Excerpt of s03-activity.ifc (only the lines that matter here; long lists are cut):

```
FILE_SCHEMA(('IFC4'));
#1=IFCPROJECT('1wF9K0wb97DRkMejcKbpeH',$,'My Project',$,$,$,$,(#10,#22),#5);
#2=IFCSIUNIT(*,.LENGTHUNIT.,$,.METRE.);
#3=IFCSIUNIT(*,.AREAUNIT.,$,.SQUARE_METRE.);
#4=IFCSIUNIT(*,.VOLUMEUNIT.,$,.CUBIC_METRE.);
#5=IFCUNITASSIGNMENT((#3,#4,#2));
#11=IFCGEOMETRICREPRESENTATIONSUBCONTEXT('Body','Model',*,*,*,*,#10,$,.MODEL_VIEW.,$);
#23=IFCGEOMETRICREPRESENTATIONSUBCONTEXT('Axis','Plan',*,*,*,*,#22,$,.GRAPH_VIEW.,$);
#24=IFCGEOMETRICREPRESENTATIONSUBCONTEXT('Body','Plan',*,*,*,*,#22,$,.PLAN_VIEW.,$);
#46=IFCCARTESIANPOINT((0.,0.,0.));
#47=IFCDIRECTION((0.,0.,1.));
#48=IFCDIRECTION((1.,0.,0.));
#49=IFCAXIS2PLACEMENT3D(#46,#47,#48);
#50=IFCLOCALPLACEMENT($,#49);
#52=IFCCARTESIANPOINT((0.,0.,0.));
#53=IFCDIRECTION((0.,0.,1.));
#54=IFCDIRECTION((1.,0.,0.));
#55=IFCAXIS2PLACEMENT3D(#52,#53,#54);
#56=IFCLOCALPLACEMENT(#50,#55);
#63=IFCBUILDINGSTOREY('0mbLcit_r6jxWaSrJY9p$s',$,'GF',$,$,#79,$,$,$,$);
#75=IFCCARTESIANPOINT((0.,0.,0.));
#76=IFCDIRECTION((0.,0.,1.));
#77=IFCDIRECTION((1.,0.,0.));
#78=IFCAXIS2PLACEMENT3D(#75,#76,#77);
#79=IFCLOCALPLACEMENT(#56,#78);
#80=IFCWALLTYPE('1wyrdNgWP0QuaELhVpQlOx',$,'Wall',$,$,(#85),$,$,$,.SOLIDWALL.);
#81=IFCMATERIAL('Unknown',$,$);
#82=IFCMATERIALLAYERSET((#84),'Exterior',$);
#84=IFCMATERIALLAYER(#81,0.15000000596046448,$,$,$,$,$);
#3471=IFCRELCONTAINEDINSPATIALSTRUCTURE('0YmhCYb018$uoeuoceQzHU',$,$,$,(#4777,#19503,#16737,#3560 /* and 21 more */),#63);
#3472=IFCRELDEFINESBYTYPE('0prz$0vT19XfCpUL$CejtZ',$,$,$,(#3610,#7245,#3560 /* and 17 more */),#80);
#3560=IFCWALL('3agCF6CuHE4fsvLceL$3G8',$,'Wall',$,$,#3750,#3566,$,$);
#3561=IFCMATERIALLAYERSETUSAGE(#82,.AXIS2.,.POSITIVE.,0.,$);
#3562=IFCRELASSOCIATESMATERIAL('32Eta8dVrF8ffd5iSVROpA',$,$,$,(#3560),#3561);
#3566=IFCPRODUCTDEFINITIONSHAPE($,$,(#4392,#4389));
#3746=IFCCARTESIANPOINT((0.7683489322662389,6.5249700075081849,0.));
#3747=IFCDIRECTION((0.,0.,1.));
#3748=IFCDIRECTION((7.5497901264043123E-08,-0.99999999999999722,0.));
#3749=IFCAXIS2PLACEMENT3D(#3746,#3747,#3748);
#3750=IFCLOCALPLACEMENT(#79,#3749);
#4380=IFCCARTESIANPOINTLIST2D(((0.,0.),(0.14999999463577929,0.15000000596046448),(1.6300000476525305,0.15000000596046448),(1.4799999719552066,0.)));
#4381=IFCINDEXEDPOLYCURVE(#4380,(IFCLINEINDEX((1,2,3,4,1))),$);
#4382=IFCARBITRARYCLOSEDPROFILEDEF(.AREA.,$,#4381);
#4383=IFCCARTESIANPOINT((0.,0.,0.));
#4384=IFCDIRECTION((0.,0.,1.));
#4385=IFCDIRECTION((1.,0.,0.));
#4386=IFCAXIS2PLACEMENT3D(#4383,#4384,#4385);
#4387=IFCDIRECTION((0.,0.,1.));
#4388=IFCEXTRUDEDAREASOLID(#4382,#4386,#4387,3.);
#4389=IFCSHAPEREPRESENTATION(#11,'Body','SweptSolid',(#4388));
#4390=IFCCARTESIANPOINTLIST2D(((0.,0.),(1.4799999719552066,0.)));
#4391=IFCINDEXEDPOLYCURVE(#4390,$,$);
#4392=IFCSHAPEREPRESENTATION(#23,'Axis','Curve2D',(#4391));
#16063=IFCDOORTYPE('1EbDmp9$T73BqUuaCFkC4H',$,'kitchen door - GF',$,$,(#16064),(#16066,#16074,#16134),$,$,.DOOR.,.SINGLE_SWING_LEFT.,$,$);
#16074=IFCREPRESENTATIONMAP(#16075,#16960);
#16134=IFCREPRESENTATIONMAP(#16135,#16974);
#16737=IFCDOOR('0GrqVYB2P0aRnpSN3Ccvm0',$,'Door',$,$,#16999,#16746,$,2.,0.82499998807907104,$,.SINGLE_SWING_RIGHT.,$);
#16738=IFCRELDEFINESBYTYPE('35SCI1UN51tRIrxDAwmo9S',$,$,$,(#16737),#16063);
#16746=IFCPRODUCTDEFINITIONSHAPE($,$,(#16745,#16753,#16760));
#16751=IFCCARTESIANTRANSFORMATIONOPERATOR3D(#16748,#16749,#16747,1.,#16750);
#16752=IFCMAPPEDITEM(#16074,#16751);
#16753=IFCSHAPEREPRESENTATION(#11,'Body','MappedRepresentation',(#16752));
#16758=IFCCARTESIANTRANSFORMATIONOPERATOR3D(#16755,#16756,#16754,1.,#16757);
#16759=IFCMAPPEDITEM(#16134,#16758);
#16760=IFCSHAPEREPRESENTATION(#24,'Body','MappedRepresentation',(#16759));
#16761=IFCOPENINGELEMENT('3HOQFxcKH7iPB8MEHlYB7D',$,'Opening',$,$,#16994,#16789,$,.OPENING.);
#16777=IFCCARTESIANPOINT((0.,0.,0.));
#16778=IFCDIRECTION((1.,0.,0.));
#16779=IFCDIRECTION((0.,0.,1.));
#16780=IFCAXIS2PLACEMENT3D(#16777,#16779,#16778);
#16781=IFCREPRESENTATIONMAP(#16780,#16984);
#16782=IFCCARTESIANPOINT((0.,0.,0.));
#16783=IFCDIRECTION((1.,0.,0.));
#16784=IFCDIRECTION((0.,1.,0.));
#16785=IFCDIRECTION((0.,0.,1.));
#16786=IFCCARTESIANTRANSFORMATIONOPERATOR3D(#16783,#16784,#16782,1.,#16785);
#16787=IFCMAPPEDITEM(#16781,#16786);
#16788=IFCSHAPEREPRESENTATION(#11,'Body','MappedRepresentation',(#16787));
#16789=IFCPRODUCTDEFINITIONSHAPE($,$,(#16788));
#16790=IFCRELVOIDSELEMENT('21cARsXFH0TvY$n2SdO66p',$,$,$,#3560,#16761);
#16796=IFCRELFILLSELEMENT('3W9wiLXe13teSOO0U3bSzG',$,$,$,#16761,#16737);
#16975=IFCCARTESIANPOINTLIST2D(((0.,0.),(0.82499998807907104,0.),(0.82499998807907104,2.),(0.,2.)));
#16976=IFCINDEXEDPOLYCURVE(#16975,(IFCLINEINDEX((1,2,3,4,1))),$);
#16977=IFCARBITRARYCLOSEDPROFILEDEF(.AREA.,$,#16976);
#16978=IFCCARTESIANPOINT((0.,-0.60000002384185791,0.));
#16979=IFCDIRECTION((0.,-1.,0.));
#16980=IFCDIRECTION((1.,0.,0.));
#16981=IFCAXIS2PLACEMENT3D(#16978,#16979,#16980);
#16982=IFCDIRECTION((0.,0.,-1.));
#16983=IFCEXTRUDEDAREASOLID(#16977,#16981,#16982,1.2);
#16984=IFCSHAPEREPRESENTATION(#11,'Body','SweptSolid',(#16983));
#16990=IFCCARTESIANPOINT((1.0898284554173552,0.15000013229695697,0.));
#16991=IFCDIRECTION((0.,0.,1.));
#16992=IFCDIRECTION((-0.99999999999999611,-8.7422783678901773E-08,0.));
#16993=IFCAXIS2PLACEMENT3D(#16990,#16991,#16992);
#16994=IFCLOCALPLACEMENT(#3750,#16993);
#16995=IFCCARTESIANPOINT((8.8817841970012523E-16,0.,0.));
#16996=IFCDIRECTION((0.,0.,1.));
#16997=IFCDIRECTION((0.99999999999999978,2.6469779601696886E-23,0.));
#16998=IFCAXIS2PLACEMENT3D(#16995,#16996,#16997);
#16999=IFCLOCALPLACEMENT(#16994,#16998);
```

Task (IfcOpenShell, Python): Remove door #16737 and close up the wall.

```python
import ifcopenshell
import ifcopenshell.api.feature
import ifcopenshell.api.root
import ifcopenshell.geom
import ifcopenshell.util.shape

model = ifcopenshell.open("s03-activity.ifc")
settings = ifcopenshell.geom.settings()


def volume(element):
    """Net volume in cubic metres, openings subtracted."""
    shape = ifcopenshell.geom.create_shape(settings, element)
    return ifcopenshell.util.shape.get_volume(shape.geometry)


door = model.by_id(16737)
opening = door.FillsVoids[0].RelatingOpeningElement
wall = opening.VoidsElements[0].RelatingBuildingElement
before = volume(wall)

ifcopenshell.api.root.remove_product(model, product=door)
ifcopenshell.api.feature.remove_feature(model, feature=opening)

after = volume(wall)

print(f"wall volume {before:.3f} -> {after:.3f} m3")

model.write("s03-activity_v2.ifc")
```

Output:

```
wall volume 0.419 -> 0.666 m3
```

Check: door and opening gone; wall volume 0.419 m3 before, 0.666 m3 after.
